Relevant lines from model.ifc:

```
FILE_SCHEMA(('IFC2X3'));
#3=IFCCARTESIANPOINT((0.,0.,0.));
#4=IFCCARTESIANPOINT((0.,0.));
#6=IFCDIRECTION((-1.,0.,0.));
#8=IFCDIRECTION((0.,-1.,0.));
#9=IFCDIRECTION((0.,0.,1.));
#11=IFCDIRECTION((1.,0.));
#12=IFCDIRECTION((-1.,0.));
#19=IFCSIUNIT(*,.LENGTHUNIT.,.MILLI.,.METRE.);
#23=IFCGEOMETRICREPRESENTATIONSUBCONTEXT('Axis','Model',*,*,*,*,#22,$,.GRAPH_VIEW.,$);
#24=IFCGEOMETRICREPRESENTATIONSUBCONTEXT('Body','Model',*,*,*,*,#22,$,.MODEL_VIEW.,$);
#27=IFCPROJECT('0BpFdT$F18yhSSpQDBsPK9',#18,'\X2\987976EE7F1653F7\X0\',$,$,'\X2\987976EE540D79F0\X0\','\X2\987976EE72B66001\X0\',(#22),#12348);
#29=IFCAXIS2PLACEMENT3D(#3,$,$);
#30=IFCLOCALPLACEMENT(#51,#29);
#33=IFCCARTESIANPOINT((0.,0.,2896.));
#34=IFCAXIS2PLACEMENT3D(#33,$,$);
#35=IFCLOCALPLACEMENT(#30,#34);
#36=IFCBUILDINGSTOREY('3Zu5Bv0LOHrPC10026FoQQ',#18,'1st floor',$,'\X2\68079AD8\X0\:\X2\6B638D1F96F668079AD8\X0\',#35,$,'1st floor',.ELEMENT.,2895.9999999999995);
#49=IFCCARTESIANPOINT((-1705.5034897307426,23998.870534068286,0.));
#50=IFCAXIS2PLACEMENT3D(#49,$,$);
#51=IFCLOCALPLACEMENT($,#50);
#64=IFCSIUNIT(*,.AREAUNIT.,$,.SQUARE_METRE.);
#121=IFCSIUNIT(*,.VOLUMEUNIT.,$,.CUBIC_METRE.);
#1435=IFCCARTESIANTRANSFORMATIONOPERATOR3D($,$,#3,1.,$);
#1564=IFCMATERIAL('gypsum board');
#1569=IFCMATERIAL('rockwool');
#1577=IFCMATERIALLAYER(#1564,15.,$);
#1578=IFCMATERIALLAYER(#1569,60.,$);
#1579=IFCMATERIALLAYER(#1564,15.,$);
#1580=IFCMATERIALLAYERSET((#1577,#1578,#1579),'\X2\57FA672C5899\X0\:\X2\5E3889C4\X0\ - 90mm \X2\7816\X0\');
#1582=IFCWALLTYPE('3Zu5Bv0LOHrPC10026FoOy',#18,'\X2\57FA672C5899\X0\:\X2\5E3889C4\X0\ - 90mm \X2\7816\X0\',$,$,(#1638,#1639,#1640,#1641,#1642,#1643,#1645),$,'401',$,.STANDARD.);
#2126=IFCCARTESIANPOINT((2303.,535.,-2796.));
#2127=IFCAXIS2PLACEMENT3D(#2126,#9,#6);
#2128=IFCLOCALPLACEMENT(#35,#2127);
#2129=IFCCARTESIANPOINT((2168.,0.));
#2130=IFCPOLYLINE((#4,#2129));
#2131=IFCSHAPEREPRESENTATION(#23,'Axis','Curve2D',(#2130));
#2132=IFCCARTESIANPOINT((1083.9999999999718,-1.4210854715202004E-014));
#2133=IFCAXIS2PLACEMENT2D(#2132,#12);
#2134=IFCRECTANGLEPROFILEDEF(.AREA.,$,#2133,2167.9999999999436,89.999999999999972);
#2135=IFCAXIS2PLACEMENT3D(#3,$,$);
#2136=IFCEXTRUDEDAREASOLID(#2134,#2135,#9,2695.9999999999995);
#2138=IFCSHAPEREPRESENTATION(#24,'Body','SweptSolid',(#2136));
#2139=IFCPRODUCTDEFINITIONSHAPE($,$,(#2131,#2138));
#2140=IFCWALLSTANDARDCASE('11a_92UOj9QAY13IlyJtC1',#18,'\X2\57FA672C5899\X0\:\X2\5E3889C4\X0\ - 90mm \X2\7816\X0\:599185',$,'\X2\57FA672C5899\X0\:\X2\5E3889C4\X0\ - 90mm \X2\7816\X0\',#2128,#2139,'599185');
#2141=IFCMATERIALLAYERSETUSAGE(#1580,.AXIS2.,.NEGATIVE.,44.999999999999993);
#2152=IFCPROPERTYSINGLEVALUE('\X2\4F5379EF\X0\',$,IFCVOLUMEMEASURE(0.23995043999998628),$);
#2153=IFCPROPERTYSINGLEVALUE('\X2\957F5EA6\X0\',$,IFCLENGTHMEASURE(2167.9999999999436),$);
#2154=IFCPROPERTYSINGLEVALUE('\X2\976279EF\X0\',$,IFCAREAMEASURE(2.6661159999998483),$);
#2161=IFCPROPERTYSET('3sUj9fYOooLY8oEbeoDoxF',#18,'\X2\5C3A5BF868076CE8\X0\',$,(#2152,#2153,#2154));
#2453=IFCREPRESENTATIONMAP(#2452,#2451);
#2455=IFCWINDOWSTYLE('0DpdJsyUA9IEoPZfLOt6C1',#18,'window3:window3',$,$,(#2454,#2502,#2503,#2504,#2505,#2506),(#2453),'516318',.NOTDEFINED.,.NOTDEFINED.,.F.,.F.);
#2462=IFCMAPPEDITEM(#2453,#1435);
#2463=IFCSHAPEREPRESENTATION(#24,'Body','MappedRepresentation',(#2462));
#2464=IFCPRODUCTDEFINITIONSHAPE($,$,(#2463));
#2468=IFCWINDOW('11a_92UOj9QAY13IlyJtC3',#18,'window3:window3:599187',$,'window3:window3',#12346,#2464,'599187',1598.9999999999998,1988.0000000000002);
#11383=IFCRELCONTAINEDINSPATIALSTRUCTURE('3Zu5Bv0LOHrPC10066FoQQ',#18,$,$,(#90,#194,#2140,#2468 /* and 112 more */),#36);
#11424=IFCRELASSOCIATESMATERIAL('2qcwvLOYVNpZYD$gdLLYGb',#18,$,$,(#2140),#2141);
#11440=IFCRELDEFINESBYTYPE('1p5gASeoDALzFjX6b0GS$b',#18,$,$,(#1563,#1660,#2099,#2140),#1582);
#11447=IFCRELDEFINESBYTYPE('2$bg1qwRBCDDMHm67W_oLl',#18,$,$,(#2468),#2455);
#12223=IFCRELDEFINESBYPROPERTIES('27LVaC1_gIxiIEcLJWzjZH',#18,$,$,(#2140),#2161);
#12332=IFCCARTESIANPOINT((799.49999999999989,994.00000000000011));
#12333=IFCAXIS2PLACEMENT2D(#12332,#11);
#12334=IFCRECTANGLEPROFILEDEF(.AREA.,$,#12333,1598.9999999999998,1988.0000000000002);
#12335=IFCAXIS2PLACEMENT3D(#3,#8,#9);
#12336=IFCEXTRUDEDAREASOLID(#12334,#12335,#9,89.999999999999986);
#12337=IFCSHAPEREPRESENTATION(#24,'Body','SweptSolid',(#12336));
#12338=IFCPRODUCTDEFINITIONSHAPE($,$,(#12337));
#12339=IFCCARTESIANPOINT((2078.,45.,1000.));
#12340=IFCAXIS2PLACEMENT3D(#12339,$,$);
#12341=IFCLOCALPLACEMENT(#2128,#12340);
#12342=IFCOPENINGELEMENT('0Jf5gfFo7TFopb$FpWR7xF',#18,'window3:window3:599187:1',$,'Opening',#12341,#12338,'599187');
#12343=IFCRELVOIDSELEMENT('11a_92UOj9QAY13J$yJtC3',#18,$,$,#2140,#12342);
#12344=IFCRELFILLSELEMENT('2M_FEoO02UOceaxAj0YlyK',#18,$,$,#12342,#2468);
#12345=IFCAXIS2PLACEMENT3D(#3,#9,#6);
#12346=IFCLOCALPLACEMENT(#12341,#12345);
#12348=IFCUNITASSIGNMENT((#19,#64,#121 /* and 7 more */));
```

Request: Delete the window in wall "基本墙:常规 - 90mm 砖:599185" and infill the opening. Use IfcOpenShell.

```python
import ifcopenshell
import ifcopenshell.api.feature
import ifcopenshell.api.pset
import ifcopenshell.api.root
import ifcopenshell.geom
import ifcopenshell.util.element
import ifcopenshell.util.shape
import ifcopenshell.util.unit

model = ifcopenshell.open("model.ifc")
area_scale = ifcopenshell.util.unit.calculate_unit_scale(model, "AREAUNIT")
volume_scale = ifcopenshell.util.unit.calculate_unit_scale(model, "VOLUMEUNIT")
settings = ifcopenshell.geom.settings()


def volume(element):
    """Net volume in cubic metres, openings subtracted."""
    shape = ifcopenshell.geom.create_shape(settings, element)
    return ifcopenshell.util.shape.get_volume(shape.geometry)


window = model.by_guid("11a_92UOj9QAY13IlyJtC3")
opening = window.FillsVoids[0].RelatingOpeningElement
wall = opening.VoidsElements[0].RelatingBuildingElement
before = volume(wall)

ifcopenshell.api.root.remove_product(model, product=window)
ifcopenshell.api.feature.remove_feature(model, feature=opening)

after = volume(wall)
thickness = 0.09  # wall thickness in metres

# Update the wall's stored quantities.
pset = model.by_id(ifcopenshell.util.element.get_pset(wall, "尺寸标注", should_inherit=False)["id"])
ifcopenshell.api.pset.edit_pset(model, pset=pset, properties={
    "体积": model.create_entity("IfcVolumeMeasure", after / volume_scale),
    "面积": model.create_entity("IfcAreaMeasure", after / thickness / area_scale),
})

print(f"wall volume {before:.3f} -> {after:.3f} m3")

model.write("model_edited.ifc")
```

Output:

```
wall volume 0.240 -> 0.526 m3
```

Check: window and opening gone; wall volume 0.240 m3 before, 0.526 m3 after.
